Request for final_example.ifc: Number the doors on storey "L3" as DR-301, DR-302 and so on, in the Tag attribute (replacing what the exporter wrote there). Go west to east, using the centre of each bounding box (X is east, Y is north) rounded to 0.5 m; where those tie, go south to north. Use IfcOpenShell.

First a look at what the model holds.

```python
import ifcopenshell
import ifcopenshell.util.element
import ifcopenshell.util.placement

model = ifcopenshell.open("final_example.ifc")
print(model.schema)
storey = next(s for s in model.by_type("IfcBuildingStorey") if s.Name == "L3")
doors = [e for e in ifcopenshell.util.element.get_decomposition(storey) if e.is_a("IfcDoor")]
for e in sorted(doors, key=lambda e: e.id()):
    origin = ifcopenshell.util.placement.get_local_placement(e.ObjectPlacement)[:3, 3]
    print(e.id(), e.Tag, e.Name, origin.round(2) + 0.0, sep=" | ")
```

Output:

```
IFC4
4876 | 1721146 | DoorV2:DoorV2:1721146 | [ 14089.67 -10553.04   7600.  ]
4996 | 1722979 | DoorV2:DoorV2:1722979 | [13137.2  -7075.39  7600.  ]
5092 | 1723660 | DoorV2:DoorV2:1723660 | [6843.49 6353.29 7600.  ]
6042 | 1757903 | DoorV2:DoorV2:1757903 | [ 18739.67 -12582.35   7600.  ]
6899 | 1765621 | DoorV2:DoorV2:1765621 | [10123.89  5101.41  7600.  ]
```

```python
import ifcopenshell
import ifcopenshell.geom
import ifcopenshell.util.element
import ifcopenshell.util.shape

model = ifcopenshell.open("final_example.ifc")
settings = ifcopenshell.geom.settings()
settings.set("use-world-coords", True)


def centre(element):
    shape = ifcopenshell.geom.create_shape(settings, element)
    return ifcopenshell.util.shape.get_bbox_centroid(shape.geometry)


storey = next(s for s in model.by_type("IfcBuildingStorey") if s.Name == "L3")
doors = [e for e in ifcopenshell.util.element.get_decomposition(storey) if e.is_a("IfcDoor")]

# Insertion points can sit at a corner or the storey origin, so sort by the geometry (in metres).
centres = {e: centre(e) for e in doors}
doors.sort(key=lambda e: (round(centres[e][0] / 0.5), centres[e][1]))

for i, e in enumerate(doors, start=1):
    number = f"DR-3{i:02d}"
    e.Tag = number
    print(e.id(), number)

model.write("final_example_v2.ifc")
```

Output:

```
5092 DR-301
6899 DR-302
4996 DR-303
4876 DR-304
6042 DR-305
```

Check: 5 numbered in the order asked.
